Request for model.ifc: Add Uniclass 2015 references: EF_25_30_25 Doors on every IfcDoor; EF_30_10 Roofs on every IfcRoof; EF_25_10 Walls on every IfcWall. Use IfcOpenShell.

First a look at what the model holds.

```python
import ifcopenshell

model = ifcopenshell.open("model.ifc")
print(model.schema)
print("classifications:", [c.Name for c in model.by_type("IfcClassification")])
for ifc_class in ("IfcDoor", "IfcRoof", "IfcStair", "IfcWall", "IfcWindow"):
    print(ifc_class, len(model.by_type(ifc_class)))
```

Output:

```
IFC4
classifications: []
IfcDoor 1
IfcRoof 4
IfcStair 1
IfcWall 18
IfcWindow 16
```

```python
import ifcopenshell
import ifcopenshell.api.classification

model = ifcopenshell.open("model.ifc")

system = ifcopenshell.api.classification.add_classification(model, classification="Uniclass 2015")

codes = {
    "IfcDoor": ("EF_25_30_25", "Doors"),
    "IfcRoof": ("EF_30_10", "Roofs"),
    "IfcWall": ("EF_25_10", "Walls"),
}
for ifc_class, (code, name) in codes.items():
    products = model.by_type(ifc_class)
    ifcopenshell.api.classification.add_reference(
        model, products=products, classification=system, identification=code, name=name
    )
    print(code, len(products))

model.write("model-out.ifc")
```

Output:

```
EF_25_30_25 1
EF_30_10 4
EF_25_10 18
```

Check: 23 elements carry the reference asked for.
